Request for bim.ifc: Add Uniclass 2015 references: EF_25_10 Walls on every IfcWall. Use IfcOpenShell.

First a look at what the model holds.

```python
import ifcopenshell

model = ifcopenshell.open("bim.ifc")
print(model.schema)
print("classifications:", [c.Name for c in model.by_type("IfcClassification")])
for ifc_class in ("IfcDoor", "IfcRoof", "IfcStair", "IfcWall", "IfcWindow"):
    print(ifc_class, len(model.by_type(ifc_class)))
```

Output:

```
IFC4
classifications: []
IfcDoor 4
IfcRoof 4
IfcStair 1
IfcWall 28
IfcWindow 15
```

```python
import ifcopenshell
import ifcopenshell.api.classification

model = ifcopenshell.open("bim.ifc")

system = ifcopenshell.api.classification.add_classification(model, classification="Uniclass 2015")

codes = {
    "IfcWall": ("EF_25_10", "Walls"),
}
for ifc_class, (code, name) in codes.items():
    products = model.by_type(ifc_class)
    ifcopenshell.api.classification.add_reference(
        model, products=products, classification=system, identification=code, name=name
    )
    print(code, len(products))

model.write("bim_v2.ifc")
```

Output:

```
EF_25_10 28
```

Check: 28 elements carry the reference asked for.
